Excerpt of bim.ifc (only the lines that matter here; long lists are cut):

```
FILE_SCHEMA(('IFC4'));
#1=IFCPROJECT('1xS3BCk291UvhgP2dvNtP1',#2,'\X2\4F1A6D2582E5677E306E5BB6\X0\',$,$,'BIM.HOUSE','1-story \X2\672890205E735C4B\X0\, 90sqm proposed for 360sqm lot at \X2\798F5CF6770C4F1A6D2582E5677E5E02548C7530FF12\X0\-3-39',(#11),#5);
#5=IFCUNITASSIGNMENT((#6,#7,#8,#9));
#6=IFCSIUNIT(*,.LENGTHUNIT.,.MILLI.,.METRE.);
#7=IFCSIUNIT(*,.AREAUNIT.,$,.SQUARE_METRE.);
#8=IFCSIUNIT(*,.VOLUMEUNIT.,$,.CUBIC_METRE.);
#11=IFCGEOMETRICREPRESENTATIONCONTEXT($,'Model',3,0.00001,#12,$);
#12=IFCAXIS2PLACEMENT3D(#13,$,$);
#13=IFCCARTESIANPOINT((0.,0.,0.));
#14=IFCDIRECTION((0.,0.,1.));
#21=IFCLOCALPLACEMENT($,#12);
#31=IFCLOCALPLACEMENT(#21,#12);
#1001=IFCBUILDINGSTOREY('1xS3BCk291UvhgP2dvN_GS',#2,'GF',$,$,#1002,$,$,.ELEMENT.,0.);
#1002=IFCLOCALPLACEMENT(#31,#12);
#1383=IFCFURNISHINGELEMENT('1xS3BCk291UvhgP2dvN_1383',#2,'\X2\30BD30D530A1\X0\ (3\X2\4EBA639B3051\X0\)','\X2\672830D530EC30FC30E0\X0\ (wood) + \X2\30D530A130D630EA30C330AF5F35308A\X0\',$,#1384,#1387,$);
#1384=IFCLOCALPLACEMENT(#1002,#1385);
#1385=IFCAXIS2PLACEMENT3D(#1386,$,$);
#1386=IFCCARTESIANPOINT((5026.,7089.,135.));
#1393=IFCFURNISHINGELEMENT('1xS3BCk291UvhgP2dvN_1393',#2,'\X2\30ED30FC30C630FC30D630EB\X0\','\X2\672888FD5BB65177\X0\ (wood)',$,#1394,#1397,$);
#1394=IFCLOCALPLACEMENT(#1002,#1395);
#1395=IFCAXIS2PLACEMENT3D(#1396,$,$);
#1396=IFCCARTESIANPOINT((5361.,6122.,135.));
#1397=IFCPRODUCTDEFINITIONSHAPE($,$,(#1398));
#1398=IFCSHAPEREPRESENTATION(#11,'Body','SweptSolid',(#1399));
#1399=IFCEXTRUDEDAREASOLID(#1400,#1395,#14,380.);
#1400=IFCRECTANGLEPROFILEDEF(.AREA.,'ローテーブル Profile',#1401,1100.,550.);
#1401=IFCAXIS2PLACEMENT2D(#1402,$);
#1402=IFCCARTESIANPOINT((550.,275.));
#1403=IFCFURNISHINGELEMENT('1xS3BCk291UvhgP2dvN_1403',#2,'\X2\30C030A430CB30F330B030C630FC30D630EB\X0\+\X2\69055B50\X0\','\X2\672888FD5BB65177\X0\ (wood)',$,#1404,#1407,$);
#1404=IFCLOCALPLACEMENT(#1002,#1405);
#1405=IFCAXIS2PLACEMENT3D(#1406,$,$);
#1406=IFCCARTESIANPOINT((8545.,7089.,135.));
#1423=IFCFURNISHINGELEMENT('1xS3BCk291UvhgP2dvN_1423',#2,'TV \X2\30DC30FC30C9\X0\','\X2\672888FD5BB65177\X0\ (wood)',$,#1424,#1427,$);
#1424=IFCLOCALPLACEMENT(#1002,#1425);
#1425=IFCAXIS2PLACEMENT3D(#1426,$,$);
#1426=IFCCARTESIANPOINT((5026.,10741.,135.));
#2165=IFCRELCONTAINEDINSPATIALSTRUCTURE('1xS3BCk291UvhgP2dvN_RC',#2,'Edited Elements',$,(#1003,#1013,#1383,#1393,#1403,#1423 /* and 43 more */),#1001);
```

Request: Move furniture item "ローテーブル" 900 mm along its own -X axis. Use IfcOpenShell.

```python
import ifcopenshell
import ifcopenshell.api.geometry
import ifcopenshell.util.placement
import ifcopenshell.util.unit

model = ifcopenshell.open("bim.ifc")
unit_scale = ifcopenshell.util.unit.calculate_unit_scale(model)

item = model.by_guid("1xS3BCk291UvhgP2dvN_1393")
matrix = ifcopenshell.util.placement.get_local_placement(item.ObjectPlacement)
matrix[:3, 3] -= matrix[:3, 0] * 0.9 / unit_scale
ifcopenshell.api.geometry.edit_object_placement(model, product=item, matrix=matrix, is_si=False)

print(ifcopenshell.util.placement.get_local_placement(item.ObjectPlacement).round(3) + 0.0)

model.write("bim_rev.ifc")
```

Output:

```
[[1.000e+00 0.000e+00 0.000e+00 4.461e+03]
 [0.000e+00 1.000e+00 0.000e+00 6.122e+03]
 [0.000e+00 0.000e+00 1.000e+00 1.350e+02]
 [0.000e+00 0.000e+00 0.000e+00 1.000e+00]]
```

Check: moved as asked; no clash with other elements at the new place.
